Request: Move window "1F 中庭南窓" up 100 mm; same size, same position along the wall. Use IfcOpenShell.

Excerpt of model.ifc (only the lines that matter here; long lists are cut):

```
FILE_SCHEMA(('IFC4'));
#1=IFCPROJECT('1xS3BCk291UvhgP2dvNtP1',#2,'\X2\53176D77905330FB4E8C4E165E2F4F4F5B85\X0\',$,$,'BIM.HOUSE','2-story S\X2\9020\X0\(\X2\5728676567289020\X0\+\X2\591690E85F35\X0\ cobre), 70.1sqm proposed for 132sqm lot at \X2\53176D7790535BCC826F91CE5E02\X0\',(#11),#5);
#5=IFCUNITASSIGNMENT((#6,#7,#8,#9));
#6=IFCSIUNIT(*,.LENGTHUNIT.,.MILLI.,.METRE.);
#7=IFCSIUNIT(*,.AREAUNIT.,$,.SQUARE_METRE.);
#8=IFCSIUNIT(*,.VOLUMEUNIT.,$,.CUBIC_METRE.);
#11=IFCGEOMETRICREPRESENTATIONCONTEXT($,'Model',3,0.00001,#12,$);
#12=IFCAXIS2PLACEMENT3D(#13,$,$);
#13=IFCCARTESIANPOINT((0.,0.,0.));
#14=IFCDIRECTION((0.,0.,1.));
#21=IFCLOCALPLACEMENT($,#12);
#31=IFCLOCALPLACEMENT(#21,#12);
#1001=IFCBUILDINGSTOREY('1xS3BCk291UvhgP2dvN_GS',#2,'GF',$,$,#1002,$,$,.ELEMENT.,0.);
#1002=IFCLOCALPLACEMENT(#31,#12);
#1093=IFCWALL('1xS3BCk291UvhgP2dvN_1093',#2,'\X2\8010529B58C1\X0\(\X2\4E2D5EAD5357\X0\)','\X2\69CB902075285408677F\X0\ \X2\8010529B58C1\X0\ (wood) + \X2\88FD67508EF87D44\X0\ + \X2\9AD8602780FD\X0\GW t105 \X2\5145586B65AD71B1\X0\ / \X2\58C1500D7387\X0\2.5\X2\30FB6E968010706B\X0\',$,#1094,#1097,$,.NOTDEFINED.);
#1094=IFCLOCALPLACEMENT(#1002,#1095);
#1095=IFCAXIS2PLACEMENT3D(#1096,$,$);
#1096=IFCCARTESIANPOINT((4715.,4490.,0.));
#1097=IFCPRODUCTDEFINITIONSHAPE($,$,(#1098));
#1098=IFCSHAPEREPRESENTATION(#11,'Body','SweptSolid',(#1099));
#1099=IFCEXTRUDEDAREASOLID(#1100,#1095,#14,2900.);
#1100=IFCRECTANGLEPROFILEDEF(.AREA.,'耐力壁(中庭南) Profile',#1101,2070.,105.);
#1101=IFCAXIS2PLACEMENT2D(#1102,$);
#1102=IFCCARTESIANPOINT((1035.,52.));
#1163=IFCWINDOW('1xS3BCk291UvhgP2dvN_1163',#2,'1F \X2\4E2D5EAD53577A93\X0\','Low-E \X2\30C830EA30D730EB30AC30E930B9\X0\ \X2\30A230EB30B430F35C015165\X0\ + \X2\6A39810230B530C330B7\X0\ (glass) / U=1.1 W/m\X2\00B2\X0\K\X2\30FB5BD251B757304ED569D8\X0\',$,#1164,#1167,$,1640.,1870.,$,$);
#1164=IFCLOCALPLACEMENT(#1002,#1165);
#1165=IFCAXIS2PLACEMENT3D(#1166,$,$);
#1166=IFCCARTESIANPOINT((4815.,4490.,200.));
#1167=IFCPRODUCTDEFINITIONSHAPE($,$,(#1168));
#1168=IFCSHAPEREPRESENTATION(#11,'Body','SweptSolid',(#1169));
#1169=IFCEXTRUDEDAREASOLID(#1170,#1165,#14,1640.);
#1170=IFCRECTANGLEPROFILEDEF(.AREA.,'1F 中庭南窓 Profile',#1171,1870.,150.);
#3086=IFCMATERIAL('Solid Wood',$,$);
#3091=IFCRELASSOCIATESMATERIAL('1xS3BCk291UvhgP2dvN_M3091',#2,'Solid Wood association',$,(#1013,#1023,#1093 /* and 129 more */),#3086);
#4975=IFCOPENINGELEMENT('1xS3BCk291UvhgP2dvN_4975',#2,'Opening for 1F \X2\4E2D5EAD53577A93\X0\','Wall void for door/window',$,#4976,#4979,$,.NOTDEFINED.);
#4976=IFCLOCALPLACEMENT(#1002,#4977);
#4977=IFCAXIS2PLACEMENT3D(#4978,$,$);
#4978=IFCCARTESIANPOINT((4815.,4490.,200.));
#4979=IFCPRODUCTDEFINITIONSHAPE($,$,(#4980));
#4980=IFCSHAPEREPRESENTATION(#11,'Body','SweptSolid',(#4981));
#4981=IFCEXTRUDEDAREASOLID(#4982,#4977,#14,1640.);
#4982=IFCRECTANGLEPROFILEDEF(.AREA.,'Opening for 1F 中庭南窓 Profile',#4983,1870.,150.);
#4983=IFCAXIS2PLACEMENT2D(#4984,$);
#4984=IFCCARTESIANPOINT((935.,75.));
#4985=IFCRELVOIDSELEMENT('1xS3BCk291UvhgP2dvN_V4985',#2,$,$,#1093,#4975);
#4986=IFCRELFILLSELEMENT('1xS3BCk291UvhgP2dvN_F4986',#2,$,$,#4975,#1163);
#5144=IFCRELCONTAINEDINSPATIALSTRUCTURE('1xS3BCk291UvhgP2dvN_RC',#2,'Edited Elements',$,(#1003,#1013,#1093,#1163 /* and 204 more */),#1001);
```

```python
import numpy as np
import ifcopenshell
import ifcopenshell.api.geometry
import ifcopenshell.util.placement
import ifcopenshell.util.unit

model = ifcopenshell.open("model.ifc")
unit_scale = ifcopenshell.util.unit.calculate_unit_scale(model)

window = model.by_guid("1xS3BCk291UvhgP2dvN_1163")
opening = window.FillsVoids[0].RelatingOpeningElement
dz = 100.0

shift = np.array([0.0, 0.0, dz])
# The window is not placed relative to its opening, so move both.
for product in (opening, window):
    matrix = ifcopenshell.util.placement.get_local_placement(product.ObjectPlacement)
    matrix[:3, 3] += shift
    ifcopenshell.api.geometry.edit_object_placement(model, product=product, matrix=matrix, is_si=False)

print(f"moved by {dz * unit_scale:+.3f} m")

model.write("model_updated.ifc")
```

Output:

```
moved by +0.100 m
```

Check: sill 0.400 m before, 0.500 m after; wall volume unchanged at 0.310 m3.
